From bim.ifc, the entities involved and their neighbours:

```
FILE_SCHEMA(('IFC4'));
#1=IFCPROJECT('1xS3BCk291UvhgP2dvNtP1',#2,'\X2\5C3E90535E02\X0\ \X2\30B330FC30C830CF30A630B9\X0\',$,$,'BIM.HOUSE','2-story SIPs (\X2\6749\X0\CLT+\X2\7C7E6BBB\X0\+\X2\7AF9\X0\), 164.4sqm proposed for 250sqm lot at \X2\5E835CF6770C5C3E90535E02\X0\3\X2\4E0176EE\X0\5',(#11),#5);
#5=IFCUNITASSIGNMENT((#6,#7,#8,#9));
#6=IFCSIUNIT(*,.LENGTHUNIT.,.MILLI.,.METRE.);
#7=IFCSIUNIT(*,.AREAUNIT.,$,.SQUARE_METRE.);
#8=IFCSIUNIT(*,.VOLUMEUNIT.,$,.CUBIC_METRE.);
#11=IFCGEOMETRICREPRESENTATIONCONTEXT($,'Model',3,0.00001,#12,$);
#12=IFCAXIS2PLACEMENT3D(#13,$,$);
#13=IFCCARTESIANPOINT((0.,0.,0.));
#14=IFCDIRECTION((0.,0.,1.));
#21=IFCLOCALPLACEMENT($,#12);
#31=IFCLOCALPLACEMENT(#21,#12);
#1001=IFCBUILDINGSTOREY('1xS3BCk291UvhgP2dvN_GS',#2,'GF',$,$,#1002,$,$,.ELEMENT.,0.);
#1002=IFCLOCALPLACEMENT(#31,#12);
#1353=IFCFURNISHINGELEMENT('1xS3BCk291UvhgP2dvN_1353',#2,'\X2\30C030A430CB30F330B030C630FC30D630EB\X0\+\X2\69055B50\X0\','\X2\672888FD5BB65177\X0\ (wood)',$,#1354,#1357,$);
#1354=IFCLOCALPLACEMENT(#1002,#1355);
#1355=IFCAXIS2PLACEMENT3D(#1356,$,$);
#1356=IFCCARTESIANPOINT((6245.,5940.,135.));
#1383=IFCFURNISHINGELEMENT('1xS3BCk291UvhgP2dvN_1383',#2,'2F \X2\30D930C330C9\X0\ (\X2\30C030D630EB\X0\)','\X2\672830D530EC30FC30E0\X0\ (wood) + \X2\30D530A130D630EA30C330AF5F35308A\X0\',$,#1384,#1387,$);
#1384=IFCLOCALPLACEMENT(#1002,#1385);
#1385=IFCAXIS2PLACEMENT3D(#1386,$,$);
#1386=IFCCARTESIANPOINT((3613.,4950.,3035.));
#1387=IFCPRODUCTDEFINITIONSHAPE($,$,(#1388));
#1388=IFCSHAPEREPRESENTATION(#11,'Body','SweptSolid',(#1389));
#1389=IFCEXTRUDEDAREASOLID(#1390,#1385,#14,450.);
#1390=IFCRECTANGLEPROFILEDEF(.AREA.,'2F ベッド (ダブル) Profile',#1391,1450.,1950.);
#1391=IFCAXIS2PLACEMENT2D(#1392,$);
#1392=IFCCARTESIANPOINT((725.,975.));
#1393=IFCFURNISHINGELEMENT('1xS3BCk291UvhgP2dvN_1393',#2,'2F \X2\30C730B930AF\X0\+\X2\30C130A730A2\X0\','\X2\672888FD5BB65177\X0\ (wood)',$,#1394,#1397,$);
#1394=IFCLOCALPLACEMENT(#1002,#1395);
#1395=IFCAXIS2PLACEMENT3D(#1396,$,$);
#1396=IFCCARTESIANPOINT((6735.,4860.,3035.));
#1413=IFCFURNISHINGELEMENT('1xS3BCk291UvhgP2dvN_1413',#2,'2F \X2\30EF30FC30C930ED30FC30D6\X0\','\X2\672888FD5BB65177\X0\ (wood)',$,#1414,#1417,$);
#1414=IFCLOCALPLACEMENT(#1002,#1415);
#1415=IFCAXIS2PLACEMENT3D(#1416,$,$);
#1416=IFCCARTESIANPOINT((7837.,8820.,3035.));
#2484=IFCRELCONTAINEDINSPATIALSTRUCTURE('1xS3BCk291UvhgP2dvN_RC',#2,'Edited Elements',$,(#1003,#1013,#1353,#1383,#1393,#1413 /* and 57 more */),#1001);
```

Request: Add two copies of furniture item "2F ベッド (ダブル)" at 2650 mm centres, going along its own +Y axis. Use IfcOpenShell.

```python
import ifcopenshell
import ifcopenshell.api.geometry
import ifcopenshell.api.root
import ifcopenshell.util.element
import ifcopenshell.util.placement
import ifcopenshell.util.unit

model = ifcopenshell.open("bim.ifc")
unit_scale = ifcopenshell.util.unit.calculate_unit_scale(model)


def reuse_history(source, copy):
    """copy_class also copies each property set's owner history, people and application; keep the originals."""
    for rel in copy.IsDefinedBy:
        if rel.is_a("IfcRelDefinesByProperties") and (history := rel.RelatingPropertyDefinition.OwnerHistory):
            rel.RelatingPropertyDefinition.OwnerHistory = source.OwnerHistory
            ifcopenshell.util.element.remove_deep2(model, history)


source = model.by_id(1383)
base = ifcopenshell.util.placement.get_local_placement(source.ObjectPlacement)
step = base[:3, 1] * 2.65 / unit_scale

for i in range(1, 3):
    copy = ifcopenshell.api.root.copy_class(model, product=source)
    copy.Representation = ifcopenshell.util.element.copy_deep(
        model, source.Representation, exclude=["IfcGeometricRepresentationContext", "IfcRepresentationMap"]
    )
    reuse_history(source, copy)
    matrix = base.copy()
    matrix[:3, 3] += i * step
    print("added at", matrix[:3, 3].round(3) + 0.0)
    ifcopenshell.api.geometry.edit_object_placement(model, product=copy, matrix=matrix, is_si=False)

model.write("bim_v2.ifc")
```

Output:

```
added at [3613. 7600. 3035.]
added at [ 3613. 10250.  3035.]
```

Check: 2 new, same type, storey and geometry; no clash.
